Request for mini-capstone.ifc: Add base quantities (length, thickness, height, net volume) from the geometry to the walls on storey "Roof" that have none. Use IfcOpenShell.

First a look at what the model holds.

```python
import ifcopenshell
import ifcopenshell.util.element
import ifcopenshell.util.unit

model = ifcopenshell.open("mini-capstone.ifc")
print(model.schema)
for unit_type in ("LENGTHUNIT", "AREAUNIT", "VOLUMEUNIT"):
    print(unit_type, ifcopenshell.util.unit.calculate_unit_scale(model, unit_type))
storey = next(s for s in model.by_type("IfcBuildingStorey") if s.Name == "Roof")
walls = [e for e in ifcopenshell.util.element.get_decomposition(storey) if e.is_a("IfcWall")]
for e in sorted(walls, key=lambda e: e.id()):
    print(e.id(), e.is_a(), e.Name, list(ifcopenshell.util.element.get_psets(e, qtos_only=True)), sep=" | ")
```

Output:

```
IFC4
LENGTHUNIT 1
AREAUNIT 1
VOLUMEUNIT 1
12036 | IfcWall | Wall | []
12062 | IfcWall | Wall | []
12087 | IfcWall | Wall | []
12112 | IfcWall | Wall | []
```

```python
import ifcopenshell
import ifcopenshell.api.pset
import ifcopenshell.geom
import ifcopenshell.util.element
import ifcopenshell.util.shape
import ifcopenshell.util.unit

model = ifcopenshell.open("mini-capstone.ifc")
unit_scale = ifcopenshell.util.unit.calculate_unit_scale(model)
volume_scale = ifcopenshell.util.unit.calculate_unit_scale(model, "VOLUMEUNIT")
settings = ifcopenshell.geom.settings()

storey = next(s for s in model.by_type("IfcBuildingStorey") if s.Name == "Roof")
walls = [e for e in ifcopenshell.util.element.get_decomposition(storey) if e.is_a("IfcWall")]

for e in sorted(walls, key=lambda e: e.id()):
    if ifcopenshell.util.element.get_psets(e, qtos_only=True, should_inherit=False):
        continue
    # Geometry comes back in metres, in the element's own axes.
    shape = ifcopenshell.geom.create_shape(settings, e)
    values = {
        "Length": ifcopenshell.util.shape.get_x(shape.geometry) / unit_scale,
        "Width": ifcopenshell.util.shape.get_y(shape.geometry) / unit_scale,
        "Height": ifcopenshell.util.shape.get_z(shape.geometry) / unit_scale,
        "NetVolume": ifcopenshell.util.shape.get_volume(shape.geometry) / volume_scale,
    }
    qto = ifcopenshell.api.pset.add_qto(model, product=e, name="Qto_WallBaseQuantities")
    ifcopenshell.api.pset.edit_qto(model, qto=qto, properties=values)
    print(e.id(), {k: round(v, 3) for k, v in values.items()})

model.write("mini-capstone_updated.ifc")
```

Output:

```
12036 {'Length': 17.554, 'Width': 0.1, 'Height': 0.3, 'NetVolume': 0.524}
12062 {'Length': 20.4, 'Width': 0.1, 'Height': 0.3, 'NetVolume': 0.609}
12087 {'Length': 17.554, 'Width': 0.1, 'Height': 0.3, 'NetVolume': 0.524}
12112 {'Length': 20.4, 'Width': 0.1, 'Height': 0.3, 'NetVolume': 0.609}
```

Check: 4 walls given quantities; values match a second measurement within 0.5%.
